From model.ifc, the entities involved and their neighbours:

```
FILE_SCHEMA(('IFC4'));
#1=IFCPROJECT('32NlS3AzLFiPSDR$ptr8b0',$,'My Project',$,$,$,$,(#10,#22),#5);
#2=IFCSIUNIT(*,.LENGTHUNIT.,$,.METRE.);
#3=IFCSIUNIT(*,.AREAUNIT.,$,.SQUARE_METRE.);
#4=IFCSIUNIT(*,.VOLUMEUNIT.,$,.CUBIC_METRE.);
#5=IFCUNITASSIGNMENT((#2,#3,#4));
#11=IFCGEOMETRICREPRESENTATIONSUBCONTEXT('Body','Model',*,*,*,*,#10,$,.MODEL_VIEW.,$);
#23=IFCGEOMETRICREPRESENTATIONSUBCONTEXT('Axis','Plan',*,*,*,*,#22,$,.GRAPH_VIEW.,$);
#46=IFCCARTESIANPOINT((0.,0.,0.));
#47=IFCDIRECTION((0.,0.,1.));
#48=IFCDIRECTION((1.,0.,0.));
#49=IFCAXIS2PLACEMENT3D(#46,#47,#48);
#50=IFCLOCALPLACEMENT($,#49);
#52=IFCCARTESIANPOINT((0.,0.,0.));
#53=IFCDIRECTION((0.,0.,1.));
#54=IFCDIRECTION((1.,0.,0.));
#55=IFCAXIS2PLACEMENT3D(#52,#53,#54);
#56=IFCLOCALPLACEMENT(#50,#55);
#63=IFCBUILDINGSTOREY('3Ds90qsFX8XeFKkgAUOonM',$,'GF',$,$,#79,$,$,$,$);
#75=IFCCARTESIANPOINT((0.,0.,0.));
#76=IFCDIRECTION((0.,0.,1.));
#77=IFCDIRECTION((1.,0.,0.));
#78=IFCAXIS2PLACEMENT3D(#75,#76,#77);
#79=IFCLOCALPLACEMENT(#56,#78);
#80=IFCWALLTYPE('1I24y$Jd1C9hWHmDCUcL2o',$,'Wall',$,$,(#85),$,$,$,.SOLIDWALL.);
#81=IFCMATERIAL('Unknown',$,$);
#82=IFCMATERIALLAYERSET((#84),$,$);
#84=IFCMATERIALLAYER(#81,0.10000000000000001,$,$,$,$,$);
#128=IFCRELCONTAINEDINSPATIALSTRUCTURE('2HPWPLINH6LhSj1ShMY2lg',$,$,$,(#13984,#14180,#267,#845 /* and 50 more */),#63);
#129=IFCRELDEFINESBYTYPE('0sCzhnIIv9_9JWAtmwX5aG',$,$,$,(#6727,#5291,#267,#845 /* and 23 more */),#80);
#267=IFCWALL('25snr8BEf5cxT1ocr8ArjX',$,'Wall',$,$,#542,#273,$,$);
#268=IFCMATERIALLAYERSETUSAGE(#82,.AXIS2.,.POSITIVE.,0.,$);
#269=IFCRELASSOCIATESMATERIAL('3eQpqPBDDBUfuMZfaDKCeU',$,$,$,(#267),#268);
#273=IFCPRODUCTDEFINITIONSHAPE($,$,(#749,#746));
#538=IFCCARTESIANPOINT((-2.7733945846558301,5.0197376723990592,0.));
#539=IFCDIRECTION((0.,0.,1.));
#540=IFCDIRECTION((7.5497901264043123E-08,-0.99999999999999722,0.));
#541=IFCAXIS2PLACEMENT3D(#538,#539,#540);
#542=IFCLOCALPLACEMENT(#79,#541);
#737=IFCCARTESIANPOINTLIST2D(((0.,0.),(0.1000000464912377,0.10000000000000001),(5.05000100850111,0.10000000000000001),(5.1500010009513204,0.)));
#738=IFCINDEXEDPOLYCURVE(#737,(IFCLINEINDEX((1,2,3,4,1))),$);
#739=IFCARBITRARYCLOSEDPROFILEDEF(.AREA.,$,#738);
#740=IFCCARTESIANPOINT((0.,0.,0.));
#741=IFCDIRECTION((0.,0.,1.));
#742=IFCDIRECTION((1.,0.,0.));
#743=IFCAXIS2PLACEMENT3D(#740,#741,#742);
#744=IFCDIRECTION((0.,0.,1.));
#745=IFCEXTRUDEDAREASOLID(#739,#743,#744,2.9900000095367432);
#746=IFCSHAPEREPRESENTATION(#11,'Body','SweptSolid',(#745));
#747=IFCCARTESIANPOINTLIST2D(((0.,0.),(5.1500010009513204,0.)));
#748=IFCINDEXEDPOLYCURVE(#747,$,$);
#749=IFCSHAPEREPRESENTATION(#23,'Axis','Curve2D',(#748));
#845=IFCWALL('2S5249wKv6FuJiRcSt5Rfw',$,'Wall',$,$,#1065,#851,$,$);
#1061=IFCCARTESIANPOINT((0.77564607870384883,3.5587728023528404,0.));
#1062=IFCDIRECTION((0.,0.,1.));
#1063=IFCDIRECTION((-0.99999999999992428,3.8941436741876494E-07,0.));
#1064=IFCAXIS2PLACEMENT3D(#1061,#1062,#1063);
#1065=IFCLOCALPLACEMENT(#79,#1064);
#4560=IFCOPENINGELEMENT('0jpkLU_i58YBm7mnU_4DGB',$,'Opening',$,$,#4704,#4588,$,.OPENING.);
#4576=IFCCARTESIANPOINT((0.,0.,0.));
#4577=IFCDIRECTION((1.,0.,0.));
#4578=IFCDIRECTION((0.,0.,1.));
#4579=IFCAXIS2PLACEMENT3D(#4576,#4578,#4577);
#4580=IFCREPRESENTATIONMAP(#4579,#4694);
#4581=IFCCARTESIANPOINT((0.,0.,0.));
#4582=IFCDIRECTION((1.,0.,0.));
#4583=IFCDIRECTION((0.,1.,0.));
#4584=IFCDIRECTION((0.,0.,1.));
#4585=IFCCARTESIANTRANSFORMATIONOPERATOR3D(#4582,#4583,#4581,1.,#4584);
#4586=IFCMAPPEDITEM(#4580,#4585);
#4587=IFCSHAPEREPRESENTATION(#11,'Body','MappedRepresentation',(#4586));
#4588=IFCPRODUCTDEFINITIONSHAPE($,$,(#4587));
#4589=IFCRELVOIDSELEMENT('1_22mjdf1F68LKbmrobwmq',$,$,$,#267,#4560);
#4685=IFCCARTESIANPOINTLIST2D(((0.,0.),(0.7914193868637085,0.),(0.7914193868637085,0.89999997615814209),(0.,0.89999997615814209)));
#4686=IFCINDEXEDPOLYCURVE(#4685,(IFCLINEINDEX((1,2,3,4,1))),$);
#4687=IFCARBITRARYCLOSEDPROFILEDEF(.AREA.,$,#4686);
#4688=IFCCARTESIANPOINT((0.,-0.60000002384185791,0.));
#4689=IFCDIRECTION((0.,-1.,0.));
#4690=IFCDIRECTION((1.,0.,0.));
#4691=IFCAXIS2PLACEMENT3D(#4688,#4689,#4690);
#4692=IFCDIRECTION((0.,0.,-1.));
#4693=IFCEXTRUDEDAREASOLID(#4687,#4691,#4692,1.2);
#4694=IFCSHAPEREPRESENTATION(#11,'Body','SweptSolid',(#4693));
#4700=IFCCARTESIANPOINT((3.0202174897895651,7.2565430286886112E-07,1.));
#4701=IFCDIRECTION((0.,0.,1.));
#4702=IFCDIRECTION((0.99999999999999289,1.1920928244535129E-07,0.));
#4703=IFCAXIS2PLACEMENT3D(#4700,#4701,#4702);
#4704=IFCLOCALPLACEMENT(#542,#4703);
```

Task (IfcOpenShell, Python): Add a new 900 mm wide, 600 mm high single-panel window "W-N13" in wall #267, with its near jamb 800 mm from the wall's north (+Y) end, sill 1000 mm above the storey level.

```python
import numpy as np
import ifcopenshell
import ifcopenshell.api.feature
import ifcopenshell.api.geometry
import ifcopenshell.api.root
import ifcopenshell.api.spatial
import ifcopenshell.geom
import ifcopenshell.util.element
import ifcopenshell.util.placement
import ifcopenshell.util.representation
import ifcopenshell.util.shape
import ifcopenshell.util.unit

model = ifcopenshell.open("model.ifc")
unit_scale = ifcopenshell.util.unit.calculate_unit_scale(model)
settings = ifcopenshell.geom.settings()


def volume(element):
    """Net volume in cubic metres, openings subtracted."""
    shape = ifcopenshell.geom.create_shape(settings, element)
    return ifcopenshell.util.shape.get_volume(shape.geometry)


wall = model.by_guid("25snr8BEf5cxT1ocr8ArjX")
storey = ifcopenshell.util.element.get_container(wall, ifc_class="IfcBuildingStorey")
context = ifcopenshell.util.representation.get_context(model, "Model", "Body", "MODEL_VIEW")
before = volume(wall)

width, height, from_end, sill = 0.9, 0.6, 0.8, 1  # metres

# The wall runs along its own X axis, and the end named is its -X end.
wall_shape = ifcopenshell.geom.create_shape(settings, wall)
x, y, z = ifcopenshell.util.shape.get_vertices(wall_shape.geometry).T
start = x.min() + from_end
face, thickness = float(y.min()), float(y.max() - y.min())
wall_matrix = ifcopenshell.util.placement.get_local_placement(wall.ObjectPlacement)
level = ifcopenshell.util.placement.get_local_placement(storey.ObjectPlacement)[2, 3]


def in_wall(x, y):
    """Placement at x, y metres in the wall's axes, at sill height."""
    matrix = wall_matrix.copy()
    matrix[:, 3] = wall_matrix @ np.array([x / unit_scale, y / unit_scale, 0.0, 1.0])
    matrix[2, 3] = level + sill / unit_scale
    return matrix


# Opening: a box that overshoots both wall faces by 50 mm.
opening = ifcopenshell.api.root.create_entity(model, ifc_class="IfcOpeningElement", predefined_type="OPENING")
box = ifcopenshell.api.geometry.add_wall_representation(
    model, context=context, length=width, height=height, thickness=thickness + 0.1
)
ifcopenshell.api.geometry.assign_representation(model, product=opening, representation=box)
ifcopenshell.api.geometry.edit_object_placement(model, product=opening, matrix=in_wall(start, face - 0.05), is_si=False)
ifcopenshell.api.feature.add_feature(model, feature=opening, element=wall)

window = ifcopenshell.api.root.create_entity(model, ifc_class="IfcWindow", name="W-N13", predefined_type="WINDOW")
window.OverallWidth, window.OverallHeight = width / unit_scale, height / unit_scale
window.PartitioningType = "SINGLE_PANEL"
body = ifcopenshell.api.geometry.add_window_representation(
    model,
    context=context,
    overall_width=window.OverallWidth,
    overall_height=window.OverallHeight,
    partition_type="SINGLE_PANEL",
)
ifcopenshell.api.geometry.assign_representation(model, product=window, representation=body)
ifcopenshell.api.spatial.assign_container(model, products=[window], relating_structure=storey)
ifcopenshell.api.feature.add_filling(model, opening=opening, element=window)

# Centre the window in the wall's thickness.
ifcopenshell.api.geometry.edit_object_placement(model, product=window, matrix=in_wall(start, face), is_si=False)
window_shape = ifcopenshell.geom.create_shape(settings, window)
depth = ifcopenshell.util.shape.get_vertices(window_shape.geometry)[:, 1]
offset = face + thickness / 2 - (depth.min() + depth.max()) / 2
ifcopenshell.api.geometry.edit_object_placement(model, product=window, matrix=in_wall(start, offset), is_si=False)

after = volume(wall)

print(f"wall volume {before:.3f} -> {after:.3f} m3")

model.write("model-out.ifc")
```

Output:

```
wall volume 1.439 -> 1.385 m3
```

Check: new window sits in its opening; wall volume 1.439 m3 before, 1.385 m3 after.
